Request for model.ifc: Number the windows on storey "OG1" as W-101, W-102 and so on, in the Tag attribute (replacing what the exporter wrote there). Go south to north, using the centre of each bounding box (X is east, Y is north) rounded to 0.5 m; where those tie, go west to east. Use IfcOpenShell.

First a look at what the model holds.

```python
import ifcopenshell
import ifcopenshell.util.element
import ifcopenshell.util.placement

model = ifcopenshell.open("model.ifc")
print(model.schema)
storey = next(s for s in model.by_type("IfcBuildingStorey") if s.Name == "OG1")
windows = [e for e in ifcopenshell.util.element.get_decomposition(storey) if e.is_a("IfcWindow")]
for e in sorted(windows, key=lambda e: e.id()):
    origin = ifcopenshell.util.placement.get_local_placement(e.ObjectPlacement)[:3, 3]
    print(e.id(), e.Tag, e.Name, origin.round(2) + 0.0, sep=" | ")
```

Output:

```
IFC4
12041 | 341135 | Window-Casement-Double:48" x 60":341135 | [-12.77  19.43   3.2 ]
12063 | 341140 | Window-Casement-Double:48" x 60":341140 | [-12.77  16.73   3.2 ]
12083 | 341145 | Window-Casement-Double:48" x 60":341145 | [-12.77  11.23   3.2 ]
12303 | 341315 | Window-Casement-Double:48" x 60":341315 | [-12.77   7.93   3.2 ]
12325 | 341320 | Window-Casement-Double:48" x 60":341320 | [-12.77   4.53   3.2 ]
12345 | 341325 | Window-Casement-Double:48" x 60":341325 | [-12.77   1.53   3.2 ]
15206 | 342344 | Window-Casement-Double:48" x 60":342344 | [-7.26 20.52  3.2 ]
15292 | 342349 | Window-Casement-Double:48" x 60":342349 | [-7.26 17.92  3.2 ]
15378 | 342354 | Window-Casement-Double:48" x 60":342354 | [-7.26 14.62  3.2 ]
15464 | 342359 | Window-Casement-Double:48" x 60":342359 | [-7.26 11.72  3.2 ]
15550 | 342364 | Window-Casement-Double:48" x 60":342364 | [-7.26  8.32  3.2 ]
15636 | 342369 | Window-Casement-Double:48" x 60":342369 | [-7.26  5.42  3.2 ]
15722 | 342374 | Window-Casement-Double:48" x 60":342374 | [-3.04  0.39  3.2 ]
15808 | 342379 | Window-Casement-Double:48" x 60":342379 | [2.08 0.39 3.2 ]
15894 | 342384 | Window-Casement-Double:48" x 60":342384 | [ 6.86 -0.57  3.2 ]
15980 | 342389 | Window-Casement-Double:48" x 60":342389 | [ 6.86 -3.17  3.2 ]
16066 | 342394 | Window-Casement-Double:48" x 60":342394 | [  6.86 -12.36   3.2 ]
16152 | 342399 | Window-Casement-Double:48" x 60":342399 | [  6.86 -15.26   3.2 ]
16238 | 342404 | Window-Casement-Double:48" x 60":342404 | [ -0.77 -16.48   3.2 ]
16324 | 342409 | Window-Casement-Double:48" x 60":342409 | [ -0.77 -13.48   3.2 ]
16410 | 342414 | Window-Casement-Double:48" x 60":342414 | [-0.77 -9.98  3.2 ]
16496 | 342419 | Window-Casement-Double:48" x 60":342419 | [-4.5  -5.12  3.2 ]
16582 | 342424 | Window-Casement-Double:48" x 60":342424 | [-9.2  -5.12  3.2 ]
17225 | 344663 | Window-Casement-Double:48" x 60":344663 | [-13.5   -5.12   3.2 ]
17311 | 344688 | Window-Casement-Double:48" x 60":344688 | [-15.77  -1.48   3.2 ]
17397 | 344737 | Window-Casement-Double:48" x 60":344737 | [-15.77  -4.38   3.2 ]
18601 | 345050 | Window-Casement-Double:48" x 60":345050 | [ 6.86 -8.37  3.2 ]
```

```python
import ifcopenshell
import ifcopenshell.geom
import ifcopenshell.util.element
import ifcopenshell.util.shape

model = ifcopenshell.open("model.ifc")
settings = ifcopenshell.geom.settings()
settings.set("use-world-coords", True)


def centre(element):
    shape = ifcopenshell.geom.create_shape(settings, element)
    return ifcopenshell.util.shape.get_bbox_centroid(shape.geometry)


storey = next(s for s in model.by_type("IfcBuildingStorey") if s.Name == "OG1")
windows = [e for e in ifcopenshell.util.element.get_decomposition(storey) if e.is_a("IfcWindow")]

# Insertion points can sit at a corner or the storey origin, so sort by the geometry (in metres).
centres = {e: centre(e) for e in windows}
windows.sort(key=lambda e: (round(centres[e][1] / 0.5), centres[e][0]))

for i, e in enumerate(windows, start=1):
    number = f"W-1{i:02d}"
    e.Tag = number
    print(e.id(), number)

model.write("model_edited.ifc")
```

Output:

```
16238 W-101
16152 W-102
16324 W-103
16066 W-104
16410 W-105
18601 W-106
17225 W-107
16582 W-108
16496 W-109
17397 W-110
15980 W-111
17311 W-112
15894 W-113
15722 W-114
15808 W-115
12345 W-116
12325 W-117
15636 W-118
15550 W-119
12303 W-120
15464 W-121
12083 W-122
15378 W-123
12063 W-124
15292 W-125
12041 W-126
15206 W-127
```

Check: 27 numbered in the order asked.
